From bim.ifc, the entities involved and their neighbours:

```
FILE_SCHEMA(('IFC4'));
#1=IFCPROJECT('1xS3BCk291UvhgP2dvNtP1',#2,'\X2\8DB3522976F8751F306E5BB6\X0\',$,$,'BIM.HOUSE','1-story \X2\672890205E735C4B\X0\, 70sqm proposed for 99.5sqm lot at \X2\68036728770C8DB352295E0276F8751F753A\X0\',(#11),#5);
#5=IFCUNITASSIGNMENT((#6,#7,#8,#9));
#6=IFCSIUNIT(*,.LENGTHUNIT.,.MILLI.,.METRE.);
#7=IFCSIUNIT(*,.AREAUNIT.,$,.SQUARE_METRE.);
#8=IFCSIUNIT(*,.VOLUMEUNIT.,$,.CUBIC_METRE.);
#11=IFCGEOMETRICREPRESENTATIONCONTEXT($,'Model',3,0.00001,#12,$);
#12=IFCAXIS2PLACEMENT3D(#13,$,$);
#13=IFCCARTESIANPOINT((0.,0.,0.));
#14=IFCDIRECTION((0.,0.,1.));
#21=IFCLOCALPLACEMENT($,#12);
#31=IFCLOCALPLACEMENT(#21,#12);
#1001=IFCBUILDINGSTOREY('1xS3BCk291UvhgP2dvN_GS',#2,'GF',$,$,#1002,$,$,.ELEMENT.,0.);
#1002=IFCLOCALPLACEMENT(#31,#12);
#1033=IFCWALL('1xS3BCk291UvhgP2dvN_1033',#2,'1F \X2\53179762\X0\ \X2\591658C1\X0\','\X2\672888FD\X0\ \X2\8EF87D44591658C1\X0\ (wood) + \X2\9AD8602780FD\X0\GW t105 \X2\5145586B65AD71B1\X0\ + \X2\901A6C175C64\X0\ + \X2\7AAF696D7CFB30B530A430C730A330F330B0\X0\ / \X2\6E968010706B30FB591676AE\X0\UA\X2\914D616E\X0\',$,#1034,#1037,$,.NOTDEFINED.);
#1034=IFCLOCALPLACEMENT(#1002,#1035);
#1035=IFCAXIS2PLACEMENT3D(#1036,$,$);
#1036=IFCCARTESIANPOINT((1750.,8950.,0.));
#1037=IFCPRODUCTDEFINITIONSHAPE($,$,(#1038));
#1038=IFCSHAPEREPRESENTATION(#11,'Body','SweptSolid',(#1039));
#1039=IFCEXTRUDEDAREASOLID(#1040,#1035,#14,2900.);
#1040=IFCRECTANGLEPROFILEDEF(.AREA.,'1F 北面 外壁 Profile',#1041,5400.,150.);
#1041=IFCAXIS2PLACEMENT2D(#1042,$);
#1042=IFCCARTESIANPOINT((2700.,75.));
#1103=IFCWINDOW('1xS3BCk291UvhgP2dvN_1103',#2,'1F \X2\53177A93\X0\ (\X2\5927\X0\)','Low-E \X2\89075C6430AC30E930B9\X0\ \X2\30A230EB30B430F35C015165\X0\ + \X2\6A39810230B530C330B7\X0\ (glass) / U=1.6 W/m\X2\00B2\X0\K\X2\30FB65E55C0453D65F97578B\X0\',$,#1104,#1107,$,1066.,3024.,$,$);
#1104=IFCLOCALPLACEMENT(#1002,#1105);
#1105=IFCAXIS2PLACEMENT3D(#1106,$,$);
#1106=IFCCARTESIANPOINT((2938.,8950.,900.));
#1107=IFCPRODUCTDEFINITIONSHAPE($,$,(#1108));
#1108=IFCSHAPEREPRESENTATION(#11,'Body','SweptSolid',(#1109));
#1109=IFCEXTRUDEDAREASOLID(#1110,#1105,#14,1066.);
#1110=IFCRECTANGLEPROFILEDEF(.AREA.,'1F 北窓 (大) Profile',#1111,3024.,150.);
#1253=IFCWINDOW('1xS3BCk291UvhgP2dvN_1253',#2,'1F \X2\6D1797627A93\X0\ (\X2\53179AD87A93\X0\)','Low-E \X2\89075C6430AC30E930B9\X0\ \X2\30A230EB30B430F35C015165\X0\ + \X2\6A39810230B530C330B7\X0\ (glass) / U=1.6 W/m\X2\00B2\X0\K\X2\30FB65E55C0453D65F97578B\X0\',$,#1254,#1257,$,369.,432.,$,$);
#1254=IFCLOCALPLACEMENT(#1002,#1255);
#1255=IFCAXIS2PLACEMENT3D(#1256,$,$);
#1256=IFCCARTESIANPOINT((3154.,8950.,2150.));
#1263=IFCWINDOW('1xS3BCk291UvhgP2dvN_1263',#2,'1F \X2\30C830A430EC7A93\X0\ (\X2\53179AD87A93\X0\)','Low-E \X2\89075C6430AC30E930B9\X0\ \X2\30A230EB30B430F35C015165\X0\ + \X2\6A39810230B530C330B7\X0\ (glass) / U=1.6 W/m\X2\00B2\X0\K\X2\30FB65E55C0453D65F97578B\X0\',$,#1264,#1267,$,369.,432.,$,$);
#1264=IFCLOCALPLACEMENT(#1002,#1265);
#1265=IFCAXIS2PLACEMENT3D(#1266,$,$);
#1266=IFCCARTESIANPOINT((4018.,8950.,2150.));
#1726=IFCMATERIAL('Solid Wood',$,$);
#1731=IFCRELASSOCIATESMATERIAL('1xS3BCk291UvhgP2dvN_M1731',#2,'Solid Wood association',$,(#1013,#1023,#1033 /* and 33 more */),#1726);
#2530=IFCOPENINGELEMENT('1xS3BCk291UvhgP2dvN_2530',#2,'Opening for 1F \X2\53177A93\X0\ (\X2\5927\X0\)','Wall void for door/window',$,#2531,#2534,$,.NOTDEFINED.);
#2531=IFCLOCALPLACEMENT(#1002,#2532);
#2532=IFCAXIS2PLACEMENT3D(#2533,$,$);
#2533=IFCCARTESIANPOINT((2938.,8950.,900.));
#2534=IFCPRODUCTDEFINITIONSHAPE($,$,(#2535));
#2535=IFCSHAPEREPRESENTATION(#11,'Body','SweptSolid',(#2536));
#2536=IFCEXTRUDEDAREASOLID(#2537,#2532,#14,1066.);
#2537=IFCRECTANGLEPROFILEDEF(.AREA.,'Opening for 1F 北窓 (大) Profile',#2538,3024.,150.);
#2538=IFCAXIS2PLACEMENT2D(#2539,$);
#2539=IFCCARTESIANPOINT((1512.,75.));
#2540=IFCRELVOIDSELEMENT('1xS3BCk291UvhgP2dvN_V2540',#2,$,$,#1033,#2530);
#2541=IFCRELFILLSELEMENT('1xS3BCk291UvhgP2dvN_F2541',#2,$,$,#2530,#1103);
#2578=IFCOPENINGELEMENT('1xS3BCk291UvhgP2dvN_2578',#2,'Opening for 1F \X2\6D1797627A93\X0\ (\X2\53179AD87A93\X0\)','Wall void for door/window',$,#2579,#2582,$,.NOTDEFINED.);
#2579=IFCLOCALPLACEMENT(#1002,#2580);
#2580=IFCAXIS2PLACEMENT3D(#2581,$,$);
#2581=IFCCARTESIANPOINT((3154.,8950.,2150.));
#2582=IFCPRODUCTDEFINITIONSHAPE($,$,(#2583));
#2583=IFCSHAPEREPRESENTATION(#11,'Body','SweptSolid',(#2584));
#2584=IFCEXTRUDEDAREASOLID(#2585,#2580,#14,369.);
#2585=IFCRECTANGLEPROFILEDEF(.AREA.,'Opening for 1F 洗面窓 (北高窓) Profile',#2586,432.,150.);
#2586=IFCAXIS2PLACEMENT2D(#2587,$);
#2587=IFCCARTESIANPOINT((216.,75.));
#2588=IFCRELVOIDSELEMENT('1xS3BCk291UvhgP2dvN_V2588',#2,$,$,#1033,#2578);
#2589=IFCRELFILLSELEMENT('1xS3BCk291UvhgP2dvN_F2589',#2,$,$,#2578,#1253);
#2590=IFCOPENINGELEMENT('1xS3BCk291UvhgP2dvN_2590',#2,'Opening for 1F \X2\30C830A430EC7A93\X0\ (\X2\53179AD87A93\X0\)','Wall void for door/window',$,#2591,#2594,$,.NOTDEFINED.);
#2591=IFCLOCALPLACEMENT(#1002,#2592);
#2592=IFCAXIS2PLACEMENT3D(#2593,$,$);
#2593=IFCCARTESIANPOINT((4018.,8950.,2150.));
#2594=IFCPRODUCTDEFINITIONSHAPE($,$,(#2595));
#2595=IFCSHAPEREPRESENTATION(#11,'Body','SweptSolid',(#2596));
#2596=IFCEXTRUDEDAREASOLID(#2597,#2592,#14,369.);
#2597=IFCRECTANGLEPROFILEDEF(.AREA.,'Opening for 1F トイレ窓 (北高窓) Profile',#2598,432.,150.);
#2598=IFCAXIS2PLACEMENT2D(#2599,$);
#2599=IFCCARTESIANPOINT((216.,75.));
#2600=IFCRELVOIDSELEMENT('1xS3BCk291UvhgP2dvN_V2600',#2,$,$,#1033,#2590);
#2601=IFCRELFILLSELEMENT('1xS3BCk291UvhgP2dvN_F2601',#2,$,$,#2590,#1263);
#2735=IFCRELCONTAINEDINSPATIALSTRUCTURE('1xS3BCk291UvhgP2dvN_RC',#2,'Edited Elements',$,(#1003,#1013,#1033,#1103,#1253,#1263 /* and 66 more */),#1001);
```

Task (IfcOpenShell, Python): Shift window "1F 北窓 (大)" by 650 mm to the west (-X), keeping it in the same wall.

```python
import ifcopenshell
import ifcopenshell.api.geometry
import ifcopenshell.util.placement
import ifcopenshell.util.unit

model = ifcopenshell.open("bim.ifc")
unit_scale = ifcopenshell.util.unit.calculate_unit_scale(model)

window = model.by_guid("1xS3BCk291UvhgP2dvN_1103")
opening = window.FillsVoids[0].RelatingOpeningElement
wall = opening.VoidsElements[0].RelatingBuildingElement

wall_matrix = ifcopenshell.util.placement.get_local_placement(wall.ObjectPlacement)
shift = wall_matrix[:3, 0] * -0.65 / unit_scale
before = ifcopenshell.util.placement.get_local_placement(window.ObjectPlacement)[:3, 3].copy()

# The window is not placed relative to its opening, so move both.
for product in (opening, window):
    matrix = ifcopenshell.util.placement.get_local_placement(product.ObjectPlacement)
    matrix[:3, 3] += shift
    ifcopenshell.api.geometry.edit_object_placement(model, product=product, matrix=matrix, is_si=False)

after = ifcopenshell.util.placement.get_local_placement(window.ObjectPlacement)[:3, 3]
print("window moved by", (after - before).round(3) + 0.0)

model.write("bim_rev.ifc")
```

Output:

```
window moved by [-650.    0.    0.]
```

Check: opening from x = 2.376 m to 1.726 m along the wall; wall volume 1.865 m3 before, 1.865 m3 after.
